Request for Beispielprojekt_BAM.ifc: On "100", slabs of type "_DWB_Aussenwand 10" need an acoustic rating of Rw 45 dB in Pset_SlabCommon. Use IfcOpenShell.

First a look at what the model holds.

```python
import ifcopenshell
import ifcopenshell.util.element

model = ifcopenshell.open("Beispielprojekt_BAM.ifc")
print(model.schema)
storey = next(s for s in model.by_type("IfcBuildingStorey") if s.Name == "100")
slabs = [e for e in ifcopenshell.util.element.get_decomposition(storey) if e.is_a("IfcSlab")]
seen = {}
for e in slabs:
    element_type = ifcopenshell.util.element.get_type(e)
    key = (element_type.Name if element_type != e and element_type else None, ifcopenshell.util.element.get_pset(e, "Pset_SlabCommon", "AcousticRating"))
    seen[key] = seen.get(key, 0) + 1
for (name, value), count in sorted(seen.items(), key=str):
    print(count, "x", name, "|", value)
```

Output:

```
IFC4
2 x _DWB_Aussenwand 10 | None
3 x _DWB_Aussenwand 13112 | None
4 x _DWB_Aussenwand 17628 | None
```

```python
import ifcopenshell
import ifcopenshell.api.pset
import ifcopenshell.util.element

model = ifcopenshell.open("Beispielprojekt_BAM.ifc")

storey = next(s for s in model.by_type("IfcBuildingStorey") if s.Name == "100")
slabs = [e for e in ifcopenshell.util.element.get_decomposition(storey) if e.is_a("IfcSlab")]

count = 0
for e in slabs:
    element_type = ifcopenshell.util.element.get_type(e)
    if element_type in (None, e) or element_type.Name != "_DWB_Aussenwand 10":
        continue
    # add_pset returns the element's existing set when there is one.
    pset = ifcopenshell.api.pset.add_pset(model, product=e, name="Pset_SlabCommon")
    ifcopenshell.api.pset.edit_pset(model, pset=pset, properties={"AcousticRating": "Rw 45 dB"})
    count += 1

print(count, "slabs updated")

model.write("Beispielprojekt_BAM_rev.ifc")
```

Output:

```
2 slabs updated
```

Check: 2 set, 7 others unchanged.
